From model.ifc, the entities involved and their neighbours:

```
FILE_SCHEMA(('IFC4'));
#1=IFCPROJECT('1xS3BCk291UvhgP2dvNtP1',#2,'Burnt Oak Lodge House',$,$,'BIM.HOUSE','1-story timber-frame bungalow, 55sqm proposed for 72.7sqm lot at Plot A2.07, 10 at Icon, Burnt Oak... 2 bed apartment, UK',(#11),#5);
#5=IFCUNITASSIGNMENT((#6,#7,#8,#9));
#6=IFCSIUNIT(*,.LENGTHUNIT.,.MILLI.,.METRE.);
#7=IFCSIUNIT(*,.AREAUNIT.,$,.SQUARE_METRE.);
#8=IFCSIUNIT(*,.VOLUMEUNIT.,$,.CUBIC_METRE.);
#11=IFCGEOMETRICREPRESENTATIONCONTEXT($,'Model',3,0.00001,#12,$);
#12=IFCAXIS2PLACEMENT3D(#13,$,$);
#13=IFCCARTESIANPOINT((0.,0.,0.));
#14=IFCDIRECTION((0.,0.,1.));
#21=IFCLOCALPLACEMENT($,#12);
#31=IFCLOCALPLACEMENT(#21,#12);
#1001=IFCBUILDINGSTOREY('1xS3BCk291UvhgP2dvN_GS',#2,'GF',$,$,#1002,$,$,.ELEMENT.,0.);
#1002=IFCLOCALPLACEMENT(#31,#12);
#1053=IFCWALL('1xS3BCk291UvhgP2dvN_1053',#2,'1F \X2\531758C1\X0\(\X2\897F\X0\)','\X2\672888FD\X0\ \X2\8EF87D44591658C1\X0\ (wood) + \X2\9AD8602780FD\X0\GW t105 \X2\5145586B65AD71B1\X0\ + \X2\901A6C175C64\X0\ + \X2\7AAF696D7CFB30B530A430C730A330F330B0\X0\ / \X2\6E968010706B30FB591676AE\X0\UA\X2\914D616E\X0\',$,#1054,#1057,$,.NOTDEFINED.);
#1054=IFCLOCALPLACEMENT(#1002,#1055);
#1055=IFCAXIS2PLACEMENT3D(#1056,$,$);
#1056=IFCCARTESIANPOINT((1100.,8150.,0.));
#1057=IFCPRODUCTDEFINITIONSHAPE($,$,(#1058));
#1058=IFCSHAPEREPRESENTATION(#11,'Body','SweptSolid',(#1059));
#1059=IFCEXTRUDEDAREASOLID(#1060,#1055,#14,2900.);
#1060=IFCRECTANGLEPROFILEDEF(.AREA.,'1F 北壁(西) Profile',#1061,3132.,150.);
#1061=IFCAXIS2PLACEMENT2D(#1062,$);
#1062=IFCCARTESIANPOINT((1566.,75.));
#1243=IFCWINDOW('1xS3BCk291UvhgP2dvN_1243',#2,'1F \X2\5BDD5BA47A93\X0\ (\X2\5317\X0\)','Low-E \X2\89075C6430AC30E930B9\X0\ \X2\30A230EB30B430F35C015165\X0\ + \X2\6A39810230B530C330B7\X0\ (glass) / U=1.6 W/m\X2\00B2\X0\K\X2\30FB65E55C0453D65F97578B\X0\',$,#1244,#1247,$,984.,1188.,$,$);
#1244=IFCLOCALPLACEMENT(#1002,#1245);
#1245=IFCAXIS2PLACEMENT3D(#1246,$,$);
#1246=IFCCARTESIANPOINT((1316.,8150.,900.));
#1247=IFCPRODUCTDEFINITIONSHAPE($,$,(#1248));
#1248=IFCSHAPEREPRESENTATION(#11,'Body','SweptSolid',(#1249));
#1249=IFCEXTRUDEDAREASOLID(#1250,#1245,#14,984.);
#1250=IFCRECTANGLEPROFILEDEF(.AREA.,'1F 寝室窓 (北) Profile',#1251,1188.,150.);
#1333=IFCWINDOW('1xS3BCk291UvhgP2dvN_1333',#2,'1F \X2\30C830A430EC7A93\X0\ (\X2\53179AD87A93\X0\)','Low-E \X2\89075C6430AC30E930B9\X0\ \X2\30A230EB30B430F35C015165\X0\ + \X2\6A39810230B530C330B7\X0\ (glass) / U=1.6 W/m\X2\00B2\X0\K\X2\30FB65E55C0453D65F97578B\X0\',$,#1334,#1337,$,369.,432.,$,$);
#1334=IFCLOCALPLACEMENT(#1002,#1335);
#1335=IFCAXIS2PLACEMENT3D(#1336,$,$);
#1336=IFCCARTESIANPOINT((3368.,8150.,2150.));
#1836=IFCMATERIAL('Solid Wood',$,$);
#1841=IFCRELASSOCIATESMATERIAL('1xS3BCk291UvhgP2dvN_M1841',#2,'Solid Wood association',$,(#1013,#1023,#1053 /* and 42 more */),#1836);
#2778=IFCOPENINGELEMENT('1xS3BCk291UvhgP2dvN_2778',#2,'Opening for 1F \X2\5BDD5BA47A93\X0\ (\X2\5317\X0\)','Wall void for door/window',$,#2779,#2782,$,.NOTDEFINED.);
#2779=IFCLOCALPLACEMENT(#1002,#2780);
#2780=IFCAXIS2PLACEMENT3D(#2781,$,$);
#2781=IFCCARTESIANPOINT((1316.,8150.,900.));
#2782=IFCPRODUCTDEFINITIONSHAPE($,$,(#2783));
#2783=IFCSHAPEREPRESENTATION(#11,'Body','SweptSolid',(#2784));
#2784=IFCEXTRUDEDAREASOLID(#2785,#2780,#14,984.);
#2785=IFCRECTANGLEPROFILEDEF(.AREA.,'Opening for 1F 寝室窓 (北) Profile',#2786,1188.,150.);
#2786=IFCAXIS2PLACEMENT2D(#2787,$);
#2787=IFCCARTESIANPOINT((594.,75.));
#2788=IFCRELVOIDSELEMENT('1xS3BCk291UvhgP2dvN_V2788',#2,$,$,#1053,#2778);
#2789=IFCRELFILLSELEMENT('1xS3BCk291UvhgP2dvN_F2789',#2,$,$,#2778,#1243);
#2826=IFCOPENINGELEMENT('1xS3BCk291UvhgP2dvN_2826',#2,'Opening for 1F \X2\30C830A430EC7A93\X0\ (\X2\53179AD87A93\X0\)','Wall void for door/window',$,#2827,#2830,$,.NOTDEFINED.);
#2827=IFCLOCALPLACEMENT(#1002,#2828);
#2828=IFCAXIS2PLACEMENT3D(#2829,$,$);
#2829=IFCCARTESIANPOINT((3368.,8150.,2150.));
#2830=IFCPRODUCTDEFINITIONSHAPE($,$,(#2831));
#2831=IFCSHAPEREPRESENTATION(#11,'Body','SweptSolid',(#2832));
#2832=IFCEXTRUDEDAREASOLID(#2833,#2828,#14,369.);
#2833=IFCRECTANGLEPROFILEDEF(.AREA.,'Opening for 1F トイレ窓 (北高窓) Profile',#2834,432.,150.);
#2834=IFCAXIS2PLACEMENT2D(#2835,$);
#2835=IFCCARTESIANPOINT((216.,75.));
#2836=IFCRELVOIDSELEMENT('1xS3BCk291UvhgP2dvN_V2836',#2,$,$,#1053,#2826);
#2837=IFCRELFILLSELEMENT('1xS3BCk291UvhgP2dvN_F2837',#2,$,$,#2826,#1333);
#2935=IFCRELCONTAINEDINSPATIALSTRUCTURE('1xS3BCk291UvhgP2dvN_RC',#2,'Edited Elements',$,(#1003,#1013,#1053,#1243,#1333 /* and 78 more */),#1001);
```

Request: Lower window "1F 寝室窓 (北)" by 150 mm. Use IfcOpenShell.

```python
import numpy as np
import ifcopenshell
import ifcopenshell.api.geometry
import ifcopenshell.util.placement
import ifcopenshell.util.unit

model = ifcopenshell.open("model.ifc")
unit_scale = ifcopenshell.util.unit.calculate_unit_scale(model)

window = model.by_id(1243)
opening = window.FillsVoids[0].RelatingOpeningElement
dz = -0.15 / unit_scale

shift = np.array([0.0, 0.0, dz])
# The window is not placed relative to its opening, so move both.
for product in (opening, window):
    matrix = ifcopenshell.util.placement.get_local_placement(product.ObjectPlacement)
    matrix[:3, 3] += shift
    ifcopenshell.api.geometry.edit_object_placement(model, product=product, matrix=matrix, is_si=False)

print(f"moved by {dz * unit_scale:+.3f} m")

model.write("model-out.ifc")
```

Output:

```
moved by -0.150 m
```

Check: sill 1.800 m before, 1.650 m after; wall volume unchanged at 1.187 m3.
